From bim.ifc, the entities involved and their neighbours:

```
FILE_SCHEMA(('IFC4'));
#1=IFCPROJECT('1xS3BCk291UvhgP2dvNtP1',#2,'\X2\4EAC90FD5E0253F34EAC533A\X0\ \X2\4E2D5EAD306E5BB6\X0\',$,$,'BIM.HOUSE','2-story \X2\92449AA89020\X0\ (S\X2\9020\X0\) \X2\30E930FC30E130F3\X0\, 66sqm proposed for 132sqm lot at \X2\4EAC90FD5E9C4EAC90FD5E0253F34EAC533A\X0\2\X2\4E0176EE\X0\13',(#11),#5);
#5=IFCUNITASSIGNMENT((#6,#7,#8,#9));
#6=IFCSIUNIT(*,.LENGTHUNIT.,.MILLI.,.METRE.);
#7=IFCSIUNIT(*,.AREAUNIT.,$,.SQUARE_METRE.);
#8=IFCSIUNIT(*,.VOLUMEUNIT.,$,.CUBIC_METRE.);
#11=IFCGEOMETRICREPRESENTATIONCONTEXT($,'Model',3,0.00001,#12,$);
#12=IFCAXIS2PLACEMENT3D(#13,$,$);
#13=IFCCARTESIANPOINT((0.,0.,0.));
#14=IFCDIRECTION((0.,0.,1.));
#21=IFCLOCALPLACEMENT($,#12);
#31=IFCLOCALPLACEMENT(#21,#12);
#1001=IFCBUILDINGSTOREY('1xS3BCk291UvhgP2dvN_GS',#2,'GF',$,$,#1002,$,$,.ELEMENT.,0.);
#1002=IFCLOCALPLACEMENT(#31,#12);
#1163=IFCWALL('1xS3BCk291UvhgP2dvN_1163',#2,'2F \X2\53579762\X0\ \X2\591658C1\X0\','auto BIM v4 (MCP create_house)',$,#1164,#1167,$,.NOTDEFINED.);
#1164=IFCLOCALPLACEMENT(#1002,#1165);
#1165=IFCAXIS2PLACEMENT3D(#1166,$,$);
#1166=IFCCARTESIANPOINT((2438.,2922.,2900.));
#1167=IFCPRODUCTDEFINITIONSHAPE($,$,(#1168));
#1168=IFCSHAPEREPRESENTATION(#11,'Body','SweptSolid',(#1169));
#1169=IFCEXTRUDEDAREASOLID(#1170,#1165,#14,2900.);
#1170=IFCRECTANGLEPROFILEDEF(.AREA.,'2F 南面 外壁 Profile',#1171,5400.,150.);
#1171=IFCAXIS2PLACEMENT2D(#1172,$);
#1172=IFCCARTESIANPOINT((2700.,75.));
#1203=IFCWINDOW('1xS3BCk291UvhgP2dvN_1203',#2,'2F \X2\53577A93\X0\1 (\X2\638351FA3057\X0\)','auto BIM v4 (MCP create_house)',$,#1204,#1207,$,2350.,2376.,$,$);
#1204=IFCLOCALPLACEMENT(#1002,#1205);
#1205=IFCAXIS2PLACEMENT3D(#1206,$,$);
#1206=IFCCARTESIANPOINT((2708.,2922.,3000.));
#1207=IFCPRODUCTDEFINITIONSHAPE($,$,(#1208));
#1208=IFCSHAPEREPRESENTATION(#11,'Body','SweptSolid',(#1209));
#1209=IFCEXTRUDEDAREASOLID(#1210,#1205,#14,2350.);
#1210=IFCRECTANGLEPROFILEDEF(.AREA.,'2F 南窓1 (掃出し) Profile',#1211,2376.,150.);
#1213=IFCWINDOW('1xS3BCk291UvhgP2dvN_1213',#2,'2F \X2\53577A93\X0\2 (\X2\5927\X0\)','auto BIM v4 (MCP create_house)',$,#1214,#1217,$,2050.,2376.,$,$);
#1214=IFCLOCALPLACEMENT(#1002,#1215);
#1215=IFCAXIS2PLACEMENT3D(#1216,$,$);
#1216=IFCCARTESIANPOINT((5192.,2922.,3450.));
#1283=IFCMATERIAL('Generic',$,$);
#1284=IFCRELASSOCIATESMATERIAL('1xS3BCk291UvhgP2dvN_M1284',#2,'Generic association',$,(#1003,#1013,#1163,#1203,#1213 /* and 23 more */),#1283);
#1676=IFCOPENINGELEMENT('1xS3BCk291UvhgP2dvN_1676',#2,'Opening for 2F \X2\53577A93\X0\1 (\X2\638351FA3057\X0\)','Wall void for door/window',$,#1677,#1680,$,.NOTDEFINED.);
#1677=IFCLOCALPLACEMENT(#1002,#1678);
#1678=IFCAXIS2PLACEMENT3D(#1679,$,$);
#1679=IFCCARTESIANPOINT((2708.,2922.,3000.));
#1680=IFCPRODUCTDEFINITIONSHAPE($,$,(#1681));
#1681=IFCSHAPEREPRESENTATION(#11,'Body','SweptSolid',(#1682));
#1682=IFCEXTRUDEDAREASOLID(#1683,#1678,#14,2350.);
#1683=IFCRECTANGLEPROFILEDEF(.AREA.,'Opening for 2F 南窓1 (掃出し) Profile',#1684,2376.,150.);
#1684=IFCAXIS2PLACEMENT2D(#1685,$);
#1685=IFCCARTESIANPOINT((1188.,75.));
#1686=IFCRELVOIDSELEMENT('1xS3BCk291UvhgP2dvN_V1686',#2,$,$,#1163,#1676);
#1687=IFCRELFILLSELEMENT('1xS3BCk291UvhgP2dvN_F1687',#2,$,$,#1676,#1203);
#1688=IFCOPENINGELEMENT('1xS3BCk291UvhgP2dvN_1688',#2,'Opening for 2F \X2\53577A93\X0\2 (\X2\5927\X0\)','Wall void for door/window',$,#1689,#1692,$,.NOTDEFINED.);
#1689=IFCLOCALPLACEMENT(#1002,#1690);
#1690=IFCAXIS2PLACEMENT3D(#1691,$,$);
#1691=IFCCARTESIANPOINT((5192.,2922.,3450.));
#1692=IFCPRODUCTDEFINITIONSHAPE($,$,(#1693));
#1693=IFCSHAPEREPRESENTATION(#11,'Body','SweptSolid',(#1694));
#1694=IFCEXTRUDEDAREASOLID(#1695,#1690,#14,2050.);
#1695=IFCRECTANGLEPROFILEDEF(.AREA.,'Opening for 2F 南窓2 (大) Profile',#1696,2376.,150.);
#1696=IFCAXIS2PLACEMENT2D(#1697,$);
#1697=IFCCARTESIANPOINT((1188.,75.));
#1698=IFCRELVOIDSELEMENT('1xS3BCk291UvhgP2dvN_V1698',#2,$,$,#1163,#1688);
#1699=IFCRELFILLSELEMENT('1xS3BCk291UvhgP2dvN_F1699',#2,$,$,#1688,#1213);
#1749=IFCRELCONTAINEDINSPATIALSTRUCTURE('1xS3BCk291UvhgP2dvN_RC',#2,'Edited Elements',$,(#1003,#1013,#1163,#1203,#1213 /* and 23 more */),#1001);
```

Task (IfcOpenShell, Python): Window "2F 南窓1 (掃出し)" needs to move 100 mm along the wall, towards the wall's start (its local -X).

```python
import ifcopenshell
import ifcopenshell.api.geometry
import ifcopenshell.util.placement
import ifcopenshell.util.unit

model = ifcopenshell.open("bim.ifc")
unit_scale = ifcopenshell.util.unit.calculate_unit_scale(model)

window = model.by_guid("1xS3BCk291UvhgP2dvN_1203")
opening = window.FillsVoids[0].RelatingOpeningElement
wall = opening.VoidsElements[0].RelatingBuildingElement

wall_matrix = ifcopenshell.util.placement.get_local_placement(wall.ObjectPlacement)
shift = wall_matrix[:3, 0] * -0.1 / unit_scale
before = ifcopenshell.util.placement.get_local_placement(window.ObjectPlacement)[:3, 3].copy()

# The window is not placed relative to its opening, so move both.
for product in (opening, window):
    matrix = ifcopenshell.util.placement.get_local_placement(product.ObjectPlacement)
    matrix[:3, 3] += shift
    ifcopenshell.api.geometry.edit_object_placement(model, product=product, matrix=matrix, is_si=False)

after = ifcopenshell.util.placement.get_local_placement(window.ObjectPlacement)[:3, 3]
print("window moved by", (after - before).round(3) + 0.0)

model.write("bim-out.ifc")
```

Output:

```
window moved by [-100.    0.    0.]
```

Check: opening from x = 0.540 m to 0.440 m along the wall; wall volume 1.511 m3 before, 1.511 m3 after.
